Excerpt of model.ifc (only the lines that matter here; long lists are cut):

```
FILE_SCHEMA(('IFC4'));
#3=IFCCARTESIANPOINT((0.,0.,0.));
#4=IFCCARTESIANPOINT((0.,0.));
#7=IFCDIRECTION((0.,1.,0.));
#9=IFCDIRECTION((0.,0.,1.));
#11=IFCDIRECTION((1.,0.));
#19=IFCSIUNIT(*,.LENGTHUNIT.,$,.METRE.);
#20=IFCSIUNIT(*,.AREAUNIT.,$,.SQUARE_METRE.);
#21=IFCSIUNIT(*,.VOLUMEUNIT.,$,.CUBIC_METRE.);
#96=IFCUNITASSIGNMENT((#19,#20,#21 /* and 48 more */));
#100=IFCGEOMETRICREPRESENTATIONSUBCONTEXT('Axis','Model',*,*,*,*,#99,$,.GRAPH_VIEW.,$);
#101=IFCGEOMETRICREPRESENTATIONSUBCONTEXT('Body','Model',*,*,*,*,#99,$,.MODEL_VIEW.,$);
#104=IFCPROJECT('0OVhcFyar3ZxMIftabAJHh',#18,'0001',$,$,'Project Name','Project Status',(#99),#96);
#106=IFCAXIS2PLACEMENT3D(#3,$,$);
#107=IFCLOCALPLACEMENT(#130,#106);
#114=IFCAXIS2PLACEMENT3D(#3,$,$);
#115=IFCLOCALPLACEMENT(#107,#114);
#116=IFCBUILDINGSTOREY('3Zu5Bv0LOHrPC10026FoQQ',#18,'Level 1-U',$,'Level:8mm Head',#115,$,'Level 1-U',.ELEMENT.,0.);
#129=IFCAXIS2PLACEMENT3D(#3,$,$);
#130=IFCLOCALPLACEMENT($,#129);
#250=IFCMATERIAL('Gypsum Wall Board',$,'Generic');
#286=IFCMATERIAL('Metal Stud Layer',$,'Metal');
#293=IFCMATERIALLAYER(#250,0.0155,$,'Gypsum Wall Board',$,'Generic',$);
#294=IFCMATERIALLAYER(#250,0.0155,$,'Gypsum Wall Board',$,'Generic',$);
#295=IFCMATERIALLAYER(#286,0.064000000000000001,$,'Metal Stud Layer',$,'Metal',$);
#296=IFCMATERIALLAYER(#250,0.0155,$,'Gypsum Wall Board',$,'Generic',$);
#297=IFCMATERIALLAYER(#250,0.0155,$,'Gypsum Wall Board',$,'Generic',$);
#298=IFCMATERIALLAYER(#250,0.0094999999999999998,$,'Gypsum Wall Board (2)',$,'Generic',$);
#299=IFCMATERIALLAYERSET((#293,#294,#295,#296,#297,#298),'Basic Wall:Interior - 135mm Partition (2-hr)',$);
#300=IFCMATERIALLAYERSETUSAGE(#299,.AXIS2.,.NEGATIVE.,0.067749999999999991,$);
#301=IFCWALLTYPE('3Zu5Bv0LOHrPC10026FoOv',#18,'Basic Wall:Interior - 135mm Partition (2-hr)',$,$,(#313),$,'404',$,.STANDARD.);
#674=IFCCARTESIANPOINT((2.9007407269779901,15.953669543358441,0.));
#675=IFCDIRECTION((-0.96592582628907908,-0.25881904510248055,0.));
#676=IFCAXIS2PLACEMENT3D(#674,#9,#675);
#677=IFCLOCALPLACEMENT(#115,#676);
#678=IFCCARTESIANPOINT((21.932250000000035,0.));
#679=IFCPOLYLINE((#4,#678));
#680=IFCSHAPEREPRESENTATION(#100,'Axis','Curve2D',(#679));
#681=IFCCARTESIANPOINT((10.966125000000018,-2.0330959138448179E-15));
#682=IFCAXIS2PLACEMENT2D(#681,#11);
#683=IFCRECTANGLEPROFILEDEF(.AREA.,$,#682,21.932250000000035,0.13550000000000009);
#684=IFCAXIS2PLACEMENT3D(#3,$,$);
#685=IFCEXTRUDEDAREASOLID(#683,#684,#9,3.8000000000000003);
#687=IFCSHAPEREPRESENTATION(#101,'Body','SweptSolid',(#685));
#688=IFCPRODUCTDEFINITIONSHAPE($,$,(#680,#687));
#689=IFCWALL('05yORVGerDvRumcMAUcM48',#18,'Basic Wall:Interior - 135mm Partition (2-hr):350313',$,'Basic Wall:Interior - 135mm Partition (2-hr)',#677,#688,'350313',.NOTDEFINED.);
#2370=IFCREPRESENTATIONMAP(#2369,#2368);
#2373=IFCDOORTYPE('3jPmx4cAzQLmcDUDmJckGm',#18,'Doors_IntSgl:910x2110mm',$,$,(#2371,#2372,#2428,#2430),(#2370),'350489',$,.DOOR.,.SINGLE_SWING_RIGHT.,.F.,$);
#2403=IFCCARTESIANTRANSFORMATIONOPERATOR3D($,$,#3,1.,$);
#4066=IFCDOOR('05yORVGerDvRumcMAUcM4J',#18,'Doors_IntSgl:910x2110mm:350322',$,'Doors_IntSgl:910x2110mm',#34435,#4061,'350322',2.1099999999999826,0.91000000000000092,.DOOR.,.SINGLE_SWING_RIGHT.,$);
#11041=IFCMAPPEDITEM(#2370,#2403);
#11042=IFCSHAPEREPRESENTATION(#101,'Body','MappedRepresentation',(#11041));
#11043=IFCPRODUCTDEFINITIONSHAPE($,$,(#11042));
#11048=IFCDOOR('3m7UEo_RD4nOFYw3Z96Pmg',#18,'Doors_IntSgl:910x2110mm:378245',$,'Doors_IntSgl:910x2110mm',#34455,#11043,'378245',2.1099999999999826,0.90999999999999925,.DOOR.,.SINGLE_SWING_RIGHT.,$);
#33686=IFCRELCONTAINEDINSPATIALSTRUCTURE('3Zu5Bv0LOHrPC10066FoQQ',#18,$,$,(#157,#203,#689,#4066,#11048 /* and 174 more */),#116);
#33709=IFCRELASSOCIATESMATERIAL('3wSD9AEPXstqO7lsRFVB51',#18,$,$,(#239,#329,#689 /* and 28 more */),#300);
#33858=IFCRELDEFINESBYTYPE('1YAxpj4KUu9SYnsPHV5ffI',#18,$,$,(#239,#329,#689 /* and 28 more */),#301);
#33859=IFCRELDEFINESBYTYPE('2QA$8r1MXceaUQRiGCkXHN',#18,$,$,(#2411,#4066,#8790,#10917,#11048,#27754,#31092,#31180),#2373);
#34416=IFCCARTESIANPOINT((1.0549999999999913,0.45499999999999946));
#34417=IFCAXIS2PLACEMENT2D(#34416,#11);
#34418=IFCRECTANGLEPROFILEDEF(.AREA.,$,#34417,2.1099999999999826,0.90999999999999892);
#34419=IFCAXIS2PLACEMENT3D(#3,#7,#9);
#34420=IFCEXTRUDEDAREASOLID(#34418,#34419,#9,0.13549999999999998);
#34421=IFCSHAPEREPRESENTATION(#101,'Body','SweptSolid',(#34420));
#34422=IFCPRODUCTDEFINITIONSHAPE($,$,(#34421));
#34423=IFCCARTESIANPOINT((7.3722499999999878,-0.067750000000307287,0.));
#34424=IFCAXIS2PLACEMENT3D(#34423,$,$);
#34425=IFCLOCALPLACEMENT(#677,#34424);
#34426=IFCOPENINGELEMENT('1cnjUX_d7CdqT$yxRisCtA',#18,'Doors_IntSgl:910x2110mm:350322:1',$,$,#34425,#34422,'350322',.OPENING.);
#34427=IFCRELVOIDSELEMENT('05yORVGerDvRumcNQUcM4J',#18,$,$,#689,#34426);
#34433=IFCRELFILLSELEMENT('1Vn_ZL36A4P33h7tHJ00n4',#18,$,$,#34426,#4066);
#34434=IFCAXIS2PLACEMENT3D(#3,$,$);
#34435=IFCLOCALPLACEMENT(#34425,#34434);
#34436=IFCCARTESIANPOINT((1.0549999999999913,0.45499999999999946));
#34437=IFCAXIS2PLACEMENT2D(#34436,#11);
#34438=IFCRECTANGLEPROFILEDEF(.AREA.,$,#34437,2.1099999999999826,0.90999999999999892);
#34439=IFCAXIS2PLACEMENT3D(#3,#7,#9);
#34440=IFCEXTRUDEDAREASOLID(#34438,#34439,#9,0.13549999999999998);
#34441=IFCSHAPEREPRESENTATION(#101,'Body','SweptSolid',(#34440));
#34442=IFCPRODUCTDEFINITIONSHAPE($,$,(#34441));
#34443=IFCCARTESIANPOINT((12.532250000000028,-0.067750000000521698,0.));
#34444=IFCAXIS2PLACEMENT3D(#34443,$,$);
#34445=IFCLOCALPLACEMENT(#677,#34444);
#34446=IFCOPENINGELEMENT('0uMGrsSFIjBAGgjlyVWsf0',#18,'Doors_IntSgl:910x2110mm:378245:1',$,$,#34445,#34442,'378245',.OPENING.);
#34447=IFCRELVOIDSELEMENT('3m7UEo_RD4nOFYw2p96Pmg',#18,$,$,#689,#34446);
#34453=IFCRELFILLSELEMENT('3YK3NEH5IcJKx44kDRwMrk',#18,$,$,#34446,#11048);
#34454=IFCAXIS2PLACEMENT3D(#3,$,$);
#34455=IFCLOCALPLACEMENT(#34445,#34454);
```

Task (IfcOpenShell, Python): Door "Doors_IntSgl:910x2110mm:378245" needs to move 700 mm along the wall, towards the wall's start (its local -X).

```python
import ifcopenshell
import ifcopenshell.api.geometry
import ifcopenshell.util.placement
import ifcopenshell.util.unit

model = ifcopenshell.open("model.ifc")
unit_scale = ifcopenshell.util.unit.calculate_unit_scale(model)

door = model.by_guid("3m7UEo_RD4nOFYw3Z96Pmg")
opening = door.FillsVoids[0].RelatingOpeningElement
wall = opening.VoidsElements[0].RelatingBuildingElement

wall_matrix = ifcopenshell.util.placement.get_local_placement(wall.ObjectPlacement)
shift = wall_matrix[:3, 0] * -0.7 / unit_scale
before = ifcopenshell.util.placement.get_local_placement(door.ObjectPlacement)[:3, 3].copy()

# The door is placed relative to its opening, so it follows when the opening moves.
matrix = ifcopenshell.util.placement.get_local_placement(opening.ObjectPlacement)
matrix[:3, 3] += shift
ifcopenshell.api.geometry.edit_object_placement(
    model, product=opening, matrix=matrix, is_si=False, should_transform_children=True
)

after = ifcopenshell.util.placement.get_local_placement(door.ObjectPlacement)[:3, 3]
print("door moved by", (after - before).round(3) + 0.0)

model.write("model-out.ifc")
```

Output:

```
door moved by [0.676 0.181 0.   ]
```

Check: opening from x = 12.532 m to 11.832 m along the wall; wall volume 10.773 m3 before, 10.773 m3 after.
